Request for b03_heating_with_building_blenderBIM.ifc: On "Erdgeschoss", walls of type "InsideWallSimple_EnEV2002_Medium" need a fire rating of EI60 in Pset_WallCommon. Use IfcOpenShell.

First a look at what the model holds.

```python
import ifcopenshell
import ifcopenshell.util.element

model = ifcopenshell.open("b03_heating_with_building_blenderBIM.ifc")
print(model.schema)
storey = next(s for s in model.by_type("IfcBuildingStorey") if s.Name == "Erdgeschoss")
walls = [e for e in ifcopenshell.util.element.get_decomposition(storey) if e.is_a("IfcWall")]
seen = {}
for e in walls:
    element_type = ifcopenshell.util.element.get_type(e)
    key = (element_type.Name if element_type != e and element_type else None, ifcopenshell.util.element.get_pset(e, "Pset_WallCommon", "FireRating"))
    seen[key] = seen.get(key, 0) + 1
for (name, value), count in sorted(seen.items(), key=str):
    print(count, "x", name, "|", value)
```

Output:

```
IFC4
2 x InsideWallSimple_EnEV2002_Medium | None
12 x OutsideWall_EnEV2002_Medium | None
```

```python
import ifcopenshell
import ifcopenshell.api.pset
import ifcopenshell.util.element

model = ifcopenshell.open("b03_heating_with_building_blenderBIM.ifc")

storey = next(s for s in model.by_type("IfcBuildingStorey") if s.Name == "Erdgeschoss")
walls = [e for e in ifcopenshell.util.element.get_decomposition(storey) if e.is_a("IfcWall")]

count = 0
for e in walls:
    element_type = ifcopenshell.util.element.get_type(e)
    if element_type in (None, e) or element_type.Name != "InsideWallSimple_EnEV2002_Medium":
        continue
    # add_pset returns the element's existing set when there is one.
    pset = ifcopenshell.api.pset.add_pset(model, product=e, name="Pset_WallCommon")
    ifcopenshell.api.pset.edit_pset(model, pset=pset, properties={"FireRating": "EI60"})
    count += 1

print(count, "walls updated")

model.write("b03_heating_with_building_blenderBIM-out.ifc")
```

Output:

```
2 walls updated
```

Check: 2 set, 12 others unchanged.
